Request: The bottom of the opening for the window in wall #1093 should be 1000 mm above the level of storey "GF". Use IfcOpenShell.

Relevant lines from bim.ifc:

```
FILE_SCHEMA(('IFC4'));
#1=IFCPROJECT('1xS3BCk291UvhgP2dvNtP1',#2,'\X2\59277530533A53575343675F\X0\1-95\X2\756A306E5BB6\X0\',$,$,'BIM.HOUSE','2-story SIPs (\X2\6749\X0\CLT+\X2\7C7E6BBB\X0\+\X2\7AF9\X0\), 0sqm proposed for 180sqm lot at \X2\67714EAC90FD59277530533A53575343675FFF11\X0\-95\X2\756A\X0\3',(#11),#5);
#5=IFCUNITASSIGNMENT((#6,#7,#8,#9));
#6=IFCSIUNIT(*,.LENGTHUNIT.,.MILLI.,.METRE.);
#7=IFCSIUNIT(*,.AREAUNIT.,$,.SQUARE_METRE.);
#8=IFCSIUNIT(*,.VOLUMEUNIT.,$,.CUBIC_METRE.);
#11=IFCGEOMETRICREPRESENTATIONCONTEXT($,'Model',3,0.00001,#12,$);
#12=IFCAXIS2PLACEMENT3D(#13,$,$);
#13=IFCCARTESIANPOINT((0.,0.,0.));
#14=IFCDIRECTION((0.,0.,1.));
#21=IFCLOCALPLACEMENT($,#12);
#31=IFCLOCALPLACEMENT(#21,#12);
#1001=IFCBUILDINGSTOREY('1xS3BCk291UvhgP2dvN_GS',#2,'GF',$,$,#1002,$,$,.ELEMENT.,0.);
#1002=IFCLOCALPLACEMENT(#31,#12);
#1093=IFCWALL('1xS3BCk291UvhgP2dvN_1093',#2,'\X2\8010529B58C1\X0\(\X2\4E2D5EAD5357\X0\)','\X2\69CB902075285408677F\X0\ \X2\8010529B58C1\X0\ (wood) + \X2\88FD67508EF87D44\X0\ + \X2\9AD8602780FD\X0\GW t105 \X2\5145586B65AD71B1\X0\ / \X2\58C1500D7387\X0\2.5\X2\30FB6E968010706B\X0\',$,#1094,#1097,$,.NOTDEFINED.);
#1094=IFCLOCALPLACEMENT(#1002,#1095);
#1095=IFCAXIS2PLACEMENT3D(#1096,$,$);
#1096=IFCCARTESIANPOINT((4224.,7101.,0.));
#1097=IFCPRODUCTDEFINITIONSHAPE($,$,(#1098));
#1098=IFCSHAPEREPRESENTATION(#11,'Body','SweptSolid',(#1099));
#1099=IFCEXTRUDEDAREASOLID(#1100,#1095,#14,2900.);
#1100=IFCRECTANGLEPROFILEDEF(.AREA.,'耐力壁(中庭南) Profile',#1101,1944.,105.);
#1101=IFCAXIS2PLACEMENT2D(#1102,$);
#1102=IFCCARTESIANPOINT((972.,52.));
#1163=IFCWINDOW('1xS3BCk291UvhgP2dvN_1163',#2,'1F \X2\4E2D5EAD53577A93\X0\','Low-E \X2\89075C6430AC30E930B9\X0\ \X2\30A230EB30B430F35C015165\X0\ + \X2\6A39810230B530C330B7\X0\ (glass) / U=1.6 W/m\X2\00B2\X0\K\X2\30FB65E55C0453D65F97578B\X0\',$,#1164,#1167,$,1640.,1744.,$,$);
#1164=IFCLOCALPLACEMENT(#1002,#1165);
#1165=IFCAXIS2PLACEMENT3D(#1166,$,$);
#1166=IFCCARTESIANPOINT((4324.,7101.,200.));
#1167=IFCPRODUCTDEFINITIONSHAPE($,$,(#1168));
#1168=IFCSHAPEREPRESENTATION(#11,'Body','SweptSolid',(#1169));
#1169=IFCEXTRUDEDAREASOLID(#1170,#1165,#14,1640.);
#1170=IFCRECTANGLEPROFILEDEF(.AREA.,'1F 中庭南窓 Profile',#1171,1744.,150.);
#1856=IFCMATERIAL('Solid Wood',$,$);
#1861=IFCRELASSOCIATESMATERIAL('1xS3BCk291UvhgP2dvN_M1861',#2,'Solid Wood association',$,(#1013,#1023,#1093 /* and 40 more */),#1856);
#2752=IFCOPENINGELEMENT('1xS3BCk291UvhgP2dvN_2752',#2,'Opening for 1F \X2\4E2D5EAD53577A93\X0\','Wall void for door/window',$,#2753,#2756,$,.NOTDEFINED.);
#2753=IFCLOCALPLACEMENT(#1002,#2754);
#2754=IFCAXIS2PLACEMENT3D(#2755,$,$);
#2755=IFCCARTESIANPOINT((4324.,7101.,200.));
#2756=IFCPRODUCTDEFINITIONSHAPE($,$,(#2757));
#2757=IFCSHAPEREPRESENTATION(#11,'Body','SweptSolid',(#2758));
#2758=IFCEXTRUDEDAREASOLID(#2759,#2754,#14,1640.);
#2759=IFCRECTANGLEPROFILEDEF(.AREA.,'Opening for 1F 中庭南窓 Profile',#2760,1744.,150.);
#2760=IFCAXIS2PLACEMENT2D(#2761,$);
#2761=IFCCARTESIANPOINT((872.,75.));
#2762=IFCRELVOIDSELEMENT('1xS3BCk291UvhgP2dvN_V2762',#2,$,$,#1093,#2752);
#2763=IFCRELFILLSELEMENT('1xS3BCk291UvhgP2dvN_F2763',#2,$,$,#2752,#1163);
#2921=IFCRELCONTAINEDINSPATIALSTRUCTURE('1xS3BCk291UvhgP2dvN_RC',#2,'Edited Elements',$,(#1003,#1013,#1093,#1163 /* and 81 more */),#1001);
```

```python
import numpy as np
import ifcopenshell
import ifcopenshell.api.geometry
import ifcopenshell.geom
import ifcopenshell.util.element
import ifcopenshell.util.placement
import ifcopenshell.util.shape
import ifcopenshell.util.unit

model = ifcopenshell.open("bim.ifc")
unit_scale = ifcopenshell.util.unit.calculate_unit_scale(model)

window = model.by_guid("1xS3BCk291UvhgP2dvN_1163")
opening = window.FillsVoids[0].RelatingOpeningElement
storey = ifcopenshell.util.element.get_container(window, ifc_class="IfcBuildingStorey")
level = ifcopenshell.util.placement.get_local_placement(storey.ObjectPlacement)[2, 3]

# The opening's origin need not be at the sill, so measure its lowest point.
shape = ifcopenshell.geom.create_shape(ifcopenshell.geom.settings(), opening)
bottom = ifcopenshell.util.shape.get_shape_bottom_elevation(shape, shape.geometry) / unit_scale
dz = level + 1 / unit_scale - bottom

shift = np.array([0.0, 0.0, dz])
# The window is not placed relative to its opening, so move both.
for product in (opening, window):
    matrix = ifcopenshell.util.placement.get_local_placement(product.ObjectPlacement)
    matrix[:3, 3] += shift
    ifcopenshell.api.geometry.edit_object_placement(model, product=product, matrix=matrix, is_si=False)

print(f"moved by {dz * unit_scale:+.3f} m")

model.write("bim-out.ifc")
```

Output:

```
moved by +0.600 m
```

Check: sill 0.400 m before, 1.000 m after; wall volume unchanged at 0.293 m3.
